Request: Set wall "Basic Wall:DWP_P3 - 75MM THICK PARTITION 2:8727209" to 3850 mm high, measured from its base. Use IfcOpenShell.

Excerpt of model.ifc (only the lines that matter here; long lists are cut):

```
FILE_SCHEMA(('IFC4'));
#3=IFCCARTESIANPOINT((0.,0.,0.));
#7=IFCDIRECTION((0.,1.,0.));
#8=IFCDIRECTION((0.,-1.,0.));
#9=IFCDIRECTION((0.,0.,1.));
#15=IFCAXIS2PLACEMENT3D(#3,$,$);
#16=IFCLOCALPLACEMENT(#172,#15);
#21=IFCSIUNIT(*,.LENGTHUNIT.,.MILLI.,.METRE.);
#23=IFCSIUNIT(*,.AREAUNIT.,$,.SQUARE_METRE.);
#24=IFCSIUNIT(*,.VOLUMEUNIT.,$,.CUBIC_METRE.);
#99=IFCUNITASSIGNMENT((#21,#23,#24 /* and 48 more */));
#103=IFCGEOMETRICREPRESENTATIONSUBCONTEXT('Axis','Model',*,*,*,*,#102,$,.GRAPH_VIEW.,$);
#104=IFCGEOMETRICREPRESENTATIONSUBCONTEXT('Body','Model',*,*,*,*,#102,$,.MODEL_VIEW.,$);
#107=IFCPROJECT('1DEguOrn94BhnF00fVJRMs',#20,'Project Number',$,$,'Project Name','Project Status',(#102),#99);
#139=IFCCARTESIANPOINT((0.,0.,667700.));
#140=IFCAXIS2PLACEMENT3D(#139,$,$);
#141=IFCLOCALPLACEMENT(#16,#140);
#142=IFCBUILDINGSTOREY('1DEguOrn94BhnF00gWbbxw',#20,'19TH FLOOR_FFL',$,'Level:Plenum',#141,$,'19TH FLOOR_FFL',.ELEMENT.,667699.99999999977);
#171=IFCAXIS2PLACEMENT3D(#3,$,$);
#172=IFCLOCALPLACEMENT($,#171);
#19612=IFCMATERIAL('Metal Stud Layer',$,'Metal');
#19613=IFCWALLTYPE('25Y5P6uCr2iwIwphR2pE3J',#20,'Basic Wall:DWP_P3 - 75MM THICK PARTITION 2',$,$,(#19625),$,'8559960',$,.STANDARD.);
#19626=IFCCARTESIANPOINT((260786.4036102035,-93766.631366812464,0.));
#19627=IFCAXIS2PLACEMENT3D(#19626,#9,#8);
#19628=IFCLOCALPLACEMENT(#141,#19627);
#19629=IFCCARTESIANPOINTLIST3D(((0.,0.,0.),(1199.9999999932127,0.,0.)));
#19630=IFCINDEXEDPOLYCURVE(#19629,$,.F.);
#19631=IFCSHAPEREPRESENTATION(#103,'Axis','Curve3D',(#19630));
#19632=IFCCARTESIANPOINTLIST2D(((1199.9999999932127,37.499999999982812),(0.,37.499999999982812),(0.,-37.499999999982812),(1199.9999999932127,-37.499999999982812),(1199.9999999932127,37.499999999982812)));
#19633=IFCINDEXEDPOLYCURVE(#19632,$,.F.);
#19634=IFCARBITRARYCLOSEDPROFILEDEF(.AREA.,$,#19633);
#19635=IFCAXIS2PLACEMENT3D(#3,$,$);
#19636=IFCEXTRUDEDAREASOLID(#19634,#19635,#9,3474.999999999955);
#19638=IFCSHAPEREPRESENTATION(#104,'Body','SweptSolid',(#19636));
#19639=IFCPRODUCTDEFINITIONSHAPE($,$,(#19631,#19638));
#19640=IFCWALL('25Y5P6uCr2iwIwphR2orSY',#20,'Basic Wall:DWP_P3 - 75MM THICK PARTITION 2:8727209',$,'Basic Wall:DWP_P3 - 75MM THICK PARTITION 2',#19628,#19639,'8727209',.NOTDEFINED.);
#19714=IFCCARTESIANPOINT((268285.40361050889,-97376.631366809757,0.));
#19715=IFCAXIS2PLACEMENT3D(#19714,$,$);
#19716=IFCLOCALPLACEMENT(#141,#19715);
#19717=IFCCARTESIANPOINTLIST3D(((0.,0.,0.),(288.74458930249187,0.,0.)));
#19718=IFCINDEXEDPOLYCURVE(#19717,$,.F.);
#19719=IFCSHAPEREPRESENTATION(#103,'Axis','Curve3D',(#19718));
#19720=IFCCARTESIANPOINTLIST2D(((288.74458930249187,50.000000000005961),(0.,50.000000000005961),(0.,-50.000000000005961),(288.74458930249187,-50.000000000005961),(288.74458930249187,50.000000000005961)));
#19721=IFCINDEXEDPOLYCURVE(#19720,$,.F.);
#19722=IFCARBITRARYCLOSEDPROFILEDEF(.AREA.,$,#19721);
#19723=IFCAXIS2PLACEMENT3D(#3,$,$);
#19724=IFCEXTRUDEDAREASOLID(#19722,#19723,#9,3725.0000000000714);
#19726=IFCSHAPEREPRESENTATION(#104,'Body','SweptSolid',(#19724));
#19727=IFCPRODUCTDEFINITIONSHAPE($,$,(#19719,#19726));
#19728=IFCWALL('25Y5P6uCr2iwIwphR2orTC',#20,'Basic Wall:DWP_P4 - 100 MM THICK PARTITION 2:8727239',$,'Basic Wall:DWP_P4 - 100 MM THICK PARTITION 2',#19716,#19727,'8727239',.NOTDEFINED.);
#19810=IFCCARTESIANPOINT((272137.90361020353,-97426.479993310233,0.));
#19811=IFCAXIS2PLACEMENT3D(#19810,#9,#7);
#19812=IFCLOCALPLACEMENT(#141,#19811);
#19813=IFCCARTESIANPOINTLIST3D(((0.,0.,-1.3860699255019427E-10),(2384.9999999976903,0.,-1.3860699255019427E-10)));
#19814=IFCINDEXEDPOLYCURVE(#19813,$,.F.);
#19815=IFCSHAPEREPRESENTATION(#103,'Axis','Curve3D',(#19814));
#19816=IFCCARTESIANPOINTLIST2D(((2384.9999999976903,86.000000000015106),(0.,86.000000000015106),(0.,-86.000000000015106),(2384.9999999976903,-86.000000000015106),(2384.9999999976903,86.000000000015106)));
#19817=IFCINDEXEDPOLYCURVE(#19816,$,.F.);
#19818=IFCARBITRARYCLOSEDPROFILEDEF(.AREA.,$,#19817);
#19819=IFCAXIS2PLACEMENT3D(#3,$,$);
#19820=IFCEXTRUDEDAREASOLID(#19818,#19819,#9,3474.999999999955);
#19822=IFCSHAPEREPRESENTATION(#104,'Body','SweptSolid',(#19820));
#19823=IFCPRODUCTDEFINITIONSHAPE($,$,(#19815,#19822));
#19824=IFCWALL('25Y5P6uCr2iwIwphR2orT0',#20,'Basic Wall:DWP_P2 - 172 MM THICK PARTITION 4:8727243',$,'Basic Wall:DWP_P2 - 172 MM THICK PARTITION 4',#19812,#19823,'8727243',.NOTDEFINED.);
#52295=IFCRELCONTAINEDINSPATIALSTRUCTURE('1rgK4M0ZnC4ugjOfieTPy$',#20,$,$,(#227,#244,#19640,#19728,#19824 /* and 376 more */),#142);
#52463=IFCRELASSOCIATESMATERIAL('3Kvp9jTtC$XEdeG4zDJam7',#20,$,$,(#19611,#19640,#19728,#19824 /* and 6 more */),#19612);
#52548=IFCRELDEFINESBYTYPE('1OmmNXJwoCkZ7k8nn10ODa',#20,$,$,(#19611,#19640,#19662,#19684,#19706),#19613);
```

```python
import ifcopenshell
import ifcopenshell.geom
import ifcopenshell.util.representation
import ifcopenshell.util.shape
import ifcopenshell.util.unit

model = ifcopenshell.open("model.ifc")
unit_scale = ifcopenshell.util.unit.calculate_unit_scale(model)
settings = ifcopenshell.geom.settings()


def volume(element):
    """Net volume in cubic metres, openings subtracted."""
    shape = ifcopenshell.geom.create_shape(settings, element)
    return ifcopenshell.util.shape.get_volume(shape.geometry)


wall = model.by_id(19640)
before = volume(wall)

body = ifcopenshell.util.representation.get_representation(wall, "Model", "Body")
solid = body.Items[0]
old_height = solid.Depth
solid.Depth = 3.85 / unit_scale
after = volume(wall)

print(f"height {old_height:g} -> {solid.Depth:g}, volume {before:.3f} -> {after:.3f} m3")

model.write("model-out.ifc")
```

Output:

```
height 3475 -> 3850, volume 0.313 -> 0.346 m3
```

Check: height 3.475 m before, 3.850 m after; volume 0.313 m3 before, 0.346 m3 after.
